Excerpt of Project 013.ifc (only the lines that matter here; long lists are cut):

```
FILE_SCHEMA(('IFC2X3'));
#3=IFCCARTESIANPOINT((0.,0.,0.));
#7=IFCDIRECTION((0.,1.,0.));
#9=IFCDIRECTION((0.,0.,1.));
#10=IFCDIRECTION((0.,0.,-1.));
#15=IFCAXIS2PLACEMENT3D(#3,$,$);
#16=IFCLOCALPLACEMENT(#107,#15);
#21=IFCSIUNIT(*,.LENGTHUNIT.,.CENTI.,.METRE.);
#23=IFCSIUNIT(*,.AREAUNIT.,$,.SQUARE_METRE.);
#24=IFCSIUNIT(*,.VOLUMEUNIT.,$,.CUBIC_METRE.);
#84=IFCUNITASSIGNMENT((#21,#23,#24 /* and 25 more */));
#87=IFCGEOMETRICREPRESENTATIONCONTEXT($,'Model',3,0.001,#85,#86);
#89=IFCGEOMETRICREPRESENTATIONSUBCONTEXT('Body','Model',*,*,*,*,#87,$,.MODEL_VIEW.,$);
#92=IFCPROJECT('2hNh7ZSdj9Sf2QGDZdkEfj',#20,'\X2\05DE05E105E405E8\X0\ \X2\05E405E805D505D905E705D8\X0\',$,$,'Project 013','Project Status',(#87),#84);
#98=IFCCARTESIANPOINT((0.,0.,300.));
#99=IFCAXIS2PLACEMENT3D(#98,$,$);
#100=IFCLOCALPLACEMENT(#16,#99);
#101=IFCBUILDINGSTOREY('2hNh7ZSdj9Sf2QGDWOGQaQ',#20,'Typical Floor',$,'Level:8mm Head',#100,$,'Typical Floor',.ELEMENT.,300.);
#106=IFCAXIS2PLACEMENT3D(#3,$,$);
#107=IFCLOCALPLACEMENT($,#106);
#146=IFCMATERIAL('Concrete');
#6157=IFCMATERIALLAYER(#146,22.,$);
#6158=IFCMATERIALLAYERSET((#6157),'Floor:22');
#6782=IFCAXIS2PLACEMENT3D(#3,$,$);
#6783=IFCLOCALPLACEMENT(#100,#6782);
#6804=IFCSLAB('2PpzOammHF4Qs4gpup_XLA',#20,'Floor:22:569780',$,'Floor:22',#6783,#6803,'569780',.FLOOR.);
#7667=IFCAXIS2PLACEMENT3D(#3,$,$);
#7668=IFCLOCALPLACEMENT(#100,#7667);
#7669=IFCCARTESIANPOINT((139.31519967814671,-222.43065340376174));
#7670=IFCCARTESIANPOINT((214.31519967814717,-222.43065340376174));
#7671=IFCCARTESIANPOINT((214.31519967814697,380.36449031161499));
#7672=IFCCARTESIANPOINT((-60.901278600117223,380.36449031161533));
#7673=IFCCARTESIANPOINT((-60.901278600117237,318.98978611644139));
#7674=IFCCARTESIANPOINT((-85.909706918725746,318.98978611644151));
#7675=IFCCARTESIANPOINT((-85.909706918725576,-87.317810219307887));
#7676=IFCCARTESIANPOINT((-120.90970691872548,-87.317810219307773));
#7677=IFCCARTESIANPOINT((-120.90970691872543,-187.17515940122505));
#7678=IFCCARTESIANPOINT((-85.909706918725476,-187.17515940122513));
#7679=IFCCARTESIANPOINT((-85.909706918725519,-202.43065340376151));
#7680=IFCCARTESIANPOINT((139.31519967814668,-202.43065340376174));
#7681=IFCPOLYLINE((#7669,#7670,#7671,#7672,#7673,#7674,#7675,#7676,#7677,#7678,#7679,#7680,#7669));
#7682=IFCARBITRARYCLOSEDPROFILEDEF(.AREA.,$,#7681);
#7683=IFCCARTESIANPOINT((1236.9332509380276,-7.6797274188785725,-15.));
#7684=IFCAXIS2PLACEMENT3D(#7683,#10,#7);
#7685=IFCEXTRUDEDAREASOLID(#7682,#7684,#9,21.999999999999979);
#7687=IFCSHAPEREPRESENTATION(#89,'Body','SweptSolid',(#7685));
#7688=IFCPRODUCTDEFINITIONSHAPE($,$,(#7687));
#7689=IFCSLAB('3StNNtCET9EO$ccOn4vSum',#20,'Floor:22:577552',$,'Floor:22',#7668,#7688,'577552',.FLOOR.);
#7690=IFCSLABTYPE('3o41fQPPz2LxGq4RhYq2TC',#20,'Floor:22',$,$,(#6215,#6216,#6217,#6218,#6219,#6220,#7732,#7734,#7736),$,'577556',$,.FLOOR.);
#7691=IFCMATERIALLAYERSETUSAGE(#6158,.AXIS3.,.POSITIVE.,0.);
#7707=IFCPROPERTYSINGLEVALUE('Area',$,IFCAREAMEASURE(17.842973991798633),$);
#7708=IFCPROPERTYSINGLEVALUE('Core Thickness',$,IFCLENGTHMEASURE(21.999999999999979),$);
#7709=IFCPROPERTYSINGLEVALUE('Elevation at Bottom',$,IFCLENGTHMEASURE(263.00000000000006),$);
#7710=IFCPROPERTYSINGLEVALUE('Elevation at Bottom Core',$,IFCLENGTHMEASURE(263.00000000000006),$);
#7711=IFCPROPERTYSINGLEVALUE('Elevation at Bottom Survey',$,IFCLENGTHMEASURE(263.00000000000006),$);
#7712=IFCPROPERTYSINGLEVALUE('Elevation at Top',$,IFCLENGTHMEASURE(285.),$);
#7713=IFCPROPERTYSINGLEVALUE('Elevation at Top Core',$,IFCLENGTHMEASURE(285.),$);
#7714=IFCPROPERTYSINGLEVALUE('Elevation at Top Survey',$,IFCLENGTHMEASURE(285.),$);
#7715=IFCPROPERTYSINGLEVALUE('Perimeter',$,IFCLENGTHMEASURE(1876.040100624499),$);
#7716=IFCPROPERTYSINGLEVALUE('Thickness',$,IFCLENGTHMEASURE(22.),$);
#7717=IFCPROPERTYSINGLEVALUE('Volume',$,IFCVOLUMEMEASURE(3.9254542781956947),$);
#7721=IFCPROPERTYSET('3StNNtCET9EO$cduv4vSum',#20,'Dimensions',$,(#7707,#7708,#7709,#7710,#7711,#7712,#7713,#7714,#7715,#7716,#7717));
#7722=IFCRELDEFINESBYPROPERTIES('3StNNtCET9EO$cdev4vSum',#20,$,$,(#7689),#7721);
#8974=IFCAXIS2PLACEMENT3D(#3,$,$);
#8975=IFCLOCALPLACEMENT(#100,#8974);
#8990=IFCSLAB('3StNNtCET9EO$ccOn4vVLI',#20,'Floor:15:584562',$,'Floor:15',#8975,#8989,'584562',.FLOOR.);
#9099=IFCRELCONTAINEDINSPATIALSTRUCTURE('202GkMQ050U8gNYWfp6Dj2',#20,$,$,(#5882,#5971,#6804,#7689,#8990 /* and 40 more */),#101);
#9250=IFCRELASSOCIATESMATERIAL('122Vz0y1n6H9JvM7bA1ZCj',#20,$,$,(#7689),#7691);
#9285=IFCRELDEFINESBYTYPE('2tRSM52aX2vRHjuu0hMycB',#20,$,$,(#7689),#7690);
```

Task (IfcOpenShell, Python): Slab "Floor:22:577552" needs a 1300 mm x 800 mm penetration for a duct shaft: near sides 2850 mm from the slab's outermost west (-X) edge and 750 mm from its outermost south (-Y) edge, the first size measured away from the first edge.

```python
import numpy as np
import ifcopenshell
import ifcopenshell.api.feature
import ifcopenshell.api.geometry
import ifcopenshell.api.pset
import ifcopenshell.api.root
import ifcopenshell.geom
import ifcopenshell.util.element
import ifcopenshell.util.placement
import ifcopenshell.util.representation
import ifcopenshell.util.shape
import ifcopenshell.util.unit

model = ifcopenshell.open("Project 013.ifc")
unit_scale = ifcopenshell.util.unit.calculate_unit_scale(model)
area_scale = ifcopenshell.util.unit.calculate_unit_scale(model, "AREAUNIT")
volume_scale = ifcopenshell.util.unit.calculate_unit_scale(model, "VOLUMEUNIT")
settings = ifcopenshell.geom.settings()


def volume(element):
    """Net volume in cubic metres, openings subtracted."""
    shape = ifcopenshell.geom.create_shape(settings, element)
    return ifcopenshell.util.shape.get_volume(shape.geometry)


slab = model.by_guid("3StNNtCET9EO$ccOn4vSum")
before = volume(slab)

# Extent in the slab's own axes, in metres. The edges named are its -X and -Y sides.
slab_shape = ifcopenshell.geom.create_shape(settings, slab)
vertices = ifcopenshell.util.shape.get_vertices(slab_shape.geometry)
x_min, y_min, bottom = vertices.min(axis=0)
top = vertices[:, 2].max()

opening = ifcopenshell.api.root.create_entity(model, ifc_class="IfcOpeningElement", name="Duct shaft opening")
context = ifcopenshell.util.representation.get_context(model, "Model", "Body", "MODEL_VIEW")
width, depth = 1.3, 0.8
outline = [(0.0, 0.0), (width, 0.0), (width, depth), (0.0, depth), (0.0, 0.0)]
# Overshoot both faces by 50 mm so the cut is clean.
shape = ifcopenshell.api.geometry.add_slab_representation(
    model, context=context, depth=top - bottom + 0.1, polyline=outline
)
ifcopenshell.api.geometry.assign_representation(model, product=opening, representation=shape)

matrix = ifcopenshell.util.placement.get_local_placement(slab.ObjectPlacement)
matrix[:, 3] = matrix @ np.append(np.array([x_min + 2.85, y_min + 0.75, bottom - 0.05]) / unit_scale, 1.0)
ifcopenshell.api.geometry.edit_object_placement(model, product=opening, matrix=matrix, is_si=False)
ifcopenshell.api.feature.add_feature(model, feature=opening, element=slab)

after = volume(slab)

# Update the slab's stored quantities.
pset = model.by_id(ifcopenshell.util.element.get_pset(slab, "Dimensions", should_inherit=False)["id"])
ifcopenshell.api.pset.edit_pset(model, pset=pset, properties={
    "Area": model.create_entity("IfcAreaMeasure", after / (top - bottom) / area_scale),
    "Volume": model.create_entity("IfcVolumeMeasure", after / volume_scale),
})

print(f"slab volume {before:.3f} -> {after:.3f} m3")

model.write("Project 013_rev.ifc")
```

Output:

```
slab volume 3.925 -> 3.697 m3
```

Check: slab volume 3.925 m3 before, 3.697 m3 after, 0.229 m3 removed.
